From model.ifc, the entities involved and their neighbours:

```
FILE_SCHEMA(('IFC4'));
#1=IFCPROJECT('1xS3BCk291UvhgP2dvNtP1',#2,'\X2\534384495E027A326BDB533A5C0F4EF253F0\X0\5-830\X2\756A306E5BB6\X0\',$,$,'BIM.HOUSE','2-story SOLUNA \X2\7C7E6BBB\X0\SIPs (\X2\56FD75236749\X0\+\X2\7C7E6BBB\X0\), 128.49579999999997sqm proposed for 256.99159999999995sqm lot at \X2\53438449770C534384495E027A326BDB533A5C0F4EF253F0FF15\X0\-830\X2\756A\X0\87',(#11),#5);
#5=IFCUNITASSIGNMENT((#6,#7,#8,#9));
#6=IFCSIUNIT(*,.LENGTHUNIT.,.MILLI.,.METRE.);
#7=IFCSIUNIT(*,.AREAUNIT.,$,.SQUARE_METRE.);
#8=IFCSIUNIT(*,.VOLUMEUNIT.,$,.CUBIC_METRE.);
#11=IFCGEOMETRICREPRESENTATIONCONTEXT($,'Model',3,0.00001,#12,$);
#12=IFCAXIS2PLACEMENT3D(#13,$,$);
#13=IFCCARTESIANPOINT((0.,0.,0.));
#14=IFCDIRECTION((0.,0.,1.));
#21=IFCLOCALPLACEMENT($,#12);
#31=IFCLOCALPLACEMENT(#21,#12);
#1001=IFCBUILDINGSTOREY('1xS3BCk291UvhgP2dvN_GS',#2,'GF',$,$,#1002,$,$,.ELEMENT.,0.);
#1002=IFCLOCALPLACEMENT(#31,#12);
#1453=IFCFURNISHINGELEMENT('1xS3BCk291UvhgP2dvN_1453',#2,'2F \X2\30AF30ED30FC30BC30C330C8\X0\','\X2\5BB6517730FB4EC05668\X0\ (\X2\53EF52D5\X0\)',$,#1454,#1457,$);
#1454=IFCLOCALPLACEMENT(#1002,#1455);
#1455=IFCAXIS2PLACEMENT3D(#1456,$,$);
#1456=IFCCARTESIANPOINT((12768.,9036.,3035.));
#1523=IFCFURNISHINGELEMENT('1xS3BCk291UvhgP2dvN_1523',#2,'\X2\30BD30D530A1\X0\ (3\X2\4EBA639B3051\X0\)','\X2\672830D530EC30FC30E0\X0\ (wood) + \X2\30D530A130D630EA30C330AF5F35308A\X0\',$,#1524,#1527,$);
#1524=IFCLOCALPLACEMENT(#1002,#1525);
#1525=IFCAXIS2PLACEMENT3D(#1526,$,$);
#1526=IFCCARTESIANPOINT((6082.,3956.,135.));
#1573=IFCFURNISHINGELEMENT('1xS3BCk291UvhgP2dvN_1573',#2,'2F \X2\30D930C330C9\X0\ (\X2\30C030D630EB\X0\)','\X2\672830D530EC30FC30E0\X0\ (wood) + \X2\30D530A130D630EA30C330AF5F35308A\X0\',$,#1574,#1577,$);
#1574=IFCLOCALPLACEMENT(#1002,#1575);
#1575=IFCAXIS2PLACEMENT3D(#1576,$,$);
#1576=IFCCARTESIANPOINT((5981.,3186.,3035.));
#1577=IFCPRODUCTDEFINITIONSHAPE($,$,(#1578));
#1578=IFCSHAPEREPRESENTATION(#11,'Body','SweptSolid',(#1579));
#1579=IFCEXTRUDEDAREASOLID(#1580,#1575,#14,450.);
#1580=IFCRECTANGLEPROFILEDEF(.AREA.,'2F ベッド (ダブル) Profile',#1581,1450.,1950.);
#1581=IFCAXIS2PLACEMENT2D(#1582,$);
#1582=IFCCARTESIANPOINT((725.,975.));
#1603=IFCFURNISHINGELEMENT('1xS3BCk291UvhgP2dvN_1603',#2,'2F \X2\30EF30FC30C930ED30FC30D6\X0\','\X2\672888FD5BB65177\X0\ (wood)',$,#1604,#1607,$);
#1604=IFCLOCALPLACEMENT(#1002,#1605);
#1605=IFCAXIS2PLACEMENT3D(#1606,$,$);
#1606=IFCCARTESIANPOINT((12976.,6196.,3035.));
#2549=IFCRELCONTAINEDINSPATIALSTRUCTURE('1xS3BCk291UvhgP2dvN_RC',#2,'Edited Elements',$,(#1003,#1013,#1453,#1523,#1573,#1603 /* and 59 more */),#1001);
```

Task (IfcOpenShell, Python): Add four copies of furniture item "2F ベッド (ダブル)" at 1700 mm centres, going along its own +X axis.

```python
import ifcopenshell
import ifcopenshell.api.geometry
import ifcopenshell.api.root
import ifcopenshell.util.element
import ifcopenshell.util.placement
import ifcopenshell.util.unit

model = ifcopenshell.open("model.ifc")
unit_scale = ifcopenshell.util.unit.calculate_unit_scale(model)


def reuse_history(source, copy):
    """copy_class also copies each property set's owner history, people and application; keep the originals."""
    for rel in copy.IsDefinedBy:
        if rel.is_a("IfcRelDefinesByProperties") and (history := rel.RelatingPropertyDefinition.OwnerHistory):
            rel.RelatingPropertyDefinition.OwnerHistory = source.OwnerHistory
            ifcopenshell.util.element.remove_deep2(model, history)


source = model.by_id(1573)
base = ifcopenshell.util.placement.get_local_placement(source.ObjectPlacement)
step = base[:3, 0] * 1.7 / unit_scale

for i in range(1, 5):
    copy = ifcopenshell.api.root.copy_class(model, product=source)
    copy.Representation = ifcopenshell.util.element.copy_deep(
        model, source.Representation, exclude=["IfcGeometricRepresentationContext", "IfcRepresentationMap"]
    )
    reuse_history(source, copy)
    matrix = base.copy()
    matrix[:3, 3] += i * step
    print("added at", matrix[:3, 3].round(3) + 0.0)
    ifcopenshell.api.geometry.edit_object_placement(model, product=copy, matrix=matrix, is_si=False)

model.write("model_rev.ifc")
```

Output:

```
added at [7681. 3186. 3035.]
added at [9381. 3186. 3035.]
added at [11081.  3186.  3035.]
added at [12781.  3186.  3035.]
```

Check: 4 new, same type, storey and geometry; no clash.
